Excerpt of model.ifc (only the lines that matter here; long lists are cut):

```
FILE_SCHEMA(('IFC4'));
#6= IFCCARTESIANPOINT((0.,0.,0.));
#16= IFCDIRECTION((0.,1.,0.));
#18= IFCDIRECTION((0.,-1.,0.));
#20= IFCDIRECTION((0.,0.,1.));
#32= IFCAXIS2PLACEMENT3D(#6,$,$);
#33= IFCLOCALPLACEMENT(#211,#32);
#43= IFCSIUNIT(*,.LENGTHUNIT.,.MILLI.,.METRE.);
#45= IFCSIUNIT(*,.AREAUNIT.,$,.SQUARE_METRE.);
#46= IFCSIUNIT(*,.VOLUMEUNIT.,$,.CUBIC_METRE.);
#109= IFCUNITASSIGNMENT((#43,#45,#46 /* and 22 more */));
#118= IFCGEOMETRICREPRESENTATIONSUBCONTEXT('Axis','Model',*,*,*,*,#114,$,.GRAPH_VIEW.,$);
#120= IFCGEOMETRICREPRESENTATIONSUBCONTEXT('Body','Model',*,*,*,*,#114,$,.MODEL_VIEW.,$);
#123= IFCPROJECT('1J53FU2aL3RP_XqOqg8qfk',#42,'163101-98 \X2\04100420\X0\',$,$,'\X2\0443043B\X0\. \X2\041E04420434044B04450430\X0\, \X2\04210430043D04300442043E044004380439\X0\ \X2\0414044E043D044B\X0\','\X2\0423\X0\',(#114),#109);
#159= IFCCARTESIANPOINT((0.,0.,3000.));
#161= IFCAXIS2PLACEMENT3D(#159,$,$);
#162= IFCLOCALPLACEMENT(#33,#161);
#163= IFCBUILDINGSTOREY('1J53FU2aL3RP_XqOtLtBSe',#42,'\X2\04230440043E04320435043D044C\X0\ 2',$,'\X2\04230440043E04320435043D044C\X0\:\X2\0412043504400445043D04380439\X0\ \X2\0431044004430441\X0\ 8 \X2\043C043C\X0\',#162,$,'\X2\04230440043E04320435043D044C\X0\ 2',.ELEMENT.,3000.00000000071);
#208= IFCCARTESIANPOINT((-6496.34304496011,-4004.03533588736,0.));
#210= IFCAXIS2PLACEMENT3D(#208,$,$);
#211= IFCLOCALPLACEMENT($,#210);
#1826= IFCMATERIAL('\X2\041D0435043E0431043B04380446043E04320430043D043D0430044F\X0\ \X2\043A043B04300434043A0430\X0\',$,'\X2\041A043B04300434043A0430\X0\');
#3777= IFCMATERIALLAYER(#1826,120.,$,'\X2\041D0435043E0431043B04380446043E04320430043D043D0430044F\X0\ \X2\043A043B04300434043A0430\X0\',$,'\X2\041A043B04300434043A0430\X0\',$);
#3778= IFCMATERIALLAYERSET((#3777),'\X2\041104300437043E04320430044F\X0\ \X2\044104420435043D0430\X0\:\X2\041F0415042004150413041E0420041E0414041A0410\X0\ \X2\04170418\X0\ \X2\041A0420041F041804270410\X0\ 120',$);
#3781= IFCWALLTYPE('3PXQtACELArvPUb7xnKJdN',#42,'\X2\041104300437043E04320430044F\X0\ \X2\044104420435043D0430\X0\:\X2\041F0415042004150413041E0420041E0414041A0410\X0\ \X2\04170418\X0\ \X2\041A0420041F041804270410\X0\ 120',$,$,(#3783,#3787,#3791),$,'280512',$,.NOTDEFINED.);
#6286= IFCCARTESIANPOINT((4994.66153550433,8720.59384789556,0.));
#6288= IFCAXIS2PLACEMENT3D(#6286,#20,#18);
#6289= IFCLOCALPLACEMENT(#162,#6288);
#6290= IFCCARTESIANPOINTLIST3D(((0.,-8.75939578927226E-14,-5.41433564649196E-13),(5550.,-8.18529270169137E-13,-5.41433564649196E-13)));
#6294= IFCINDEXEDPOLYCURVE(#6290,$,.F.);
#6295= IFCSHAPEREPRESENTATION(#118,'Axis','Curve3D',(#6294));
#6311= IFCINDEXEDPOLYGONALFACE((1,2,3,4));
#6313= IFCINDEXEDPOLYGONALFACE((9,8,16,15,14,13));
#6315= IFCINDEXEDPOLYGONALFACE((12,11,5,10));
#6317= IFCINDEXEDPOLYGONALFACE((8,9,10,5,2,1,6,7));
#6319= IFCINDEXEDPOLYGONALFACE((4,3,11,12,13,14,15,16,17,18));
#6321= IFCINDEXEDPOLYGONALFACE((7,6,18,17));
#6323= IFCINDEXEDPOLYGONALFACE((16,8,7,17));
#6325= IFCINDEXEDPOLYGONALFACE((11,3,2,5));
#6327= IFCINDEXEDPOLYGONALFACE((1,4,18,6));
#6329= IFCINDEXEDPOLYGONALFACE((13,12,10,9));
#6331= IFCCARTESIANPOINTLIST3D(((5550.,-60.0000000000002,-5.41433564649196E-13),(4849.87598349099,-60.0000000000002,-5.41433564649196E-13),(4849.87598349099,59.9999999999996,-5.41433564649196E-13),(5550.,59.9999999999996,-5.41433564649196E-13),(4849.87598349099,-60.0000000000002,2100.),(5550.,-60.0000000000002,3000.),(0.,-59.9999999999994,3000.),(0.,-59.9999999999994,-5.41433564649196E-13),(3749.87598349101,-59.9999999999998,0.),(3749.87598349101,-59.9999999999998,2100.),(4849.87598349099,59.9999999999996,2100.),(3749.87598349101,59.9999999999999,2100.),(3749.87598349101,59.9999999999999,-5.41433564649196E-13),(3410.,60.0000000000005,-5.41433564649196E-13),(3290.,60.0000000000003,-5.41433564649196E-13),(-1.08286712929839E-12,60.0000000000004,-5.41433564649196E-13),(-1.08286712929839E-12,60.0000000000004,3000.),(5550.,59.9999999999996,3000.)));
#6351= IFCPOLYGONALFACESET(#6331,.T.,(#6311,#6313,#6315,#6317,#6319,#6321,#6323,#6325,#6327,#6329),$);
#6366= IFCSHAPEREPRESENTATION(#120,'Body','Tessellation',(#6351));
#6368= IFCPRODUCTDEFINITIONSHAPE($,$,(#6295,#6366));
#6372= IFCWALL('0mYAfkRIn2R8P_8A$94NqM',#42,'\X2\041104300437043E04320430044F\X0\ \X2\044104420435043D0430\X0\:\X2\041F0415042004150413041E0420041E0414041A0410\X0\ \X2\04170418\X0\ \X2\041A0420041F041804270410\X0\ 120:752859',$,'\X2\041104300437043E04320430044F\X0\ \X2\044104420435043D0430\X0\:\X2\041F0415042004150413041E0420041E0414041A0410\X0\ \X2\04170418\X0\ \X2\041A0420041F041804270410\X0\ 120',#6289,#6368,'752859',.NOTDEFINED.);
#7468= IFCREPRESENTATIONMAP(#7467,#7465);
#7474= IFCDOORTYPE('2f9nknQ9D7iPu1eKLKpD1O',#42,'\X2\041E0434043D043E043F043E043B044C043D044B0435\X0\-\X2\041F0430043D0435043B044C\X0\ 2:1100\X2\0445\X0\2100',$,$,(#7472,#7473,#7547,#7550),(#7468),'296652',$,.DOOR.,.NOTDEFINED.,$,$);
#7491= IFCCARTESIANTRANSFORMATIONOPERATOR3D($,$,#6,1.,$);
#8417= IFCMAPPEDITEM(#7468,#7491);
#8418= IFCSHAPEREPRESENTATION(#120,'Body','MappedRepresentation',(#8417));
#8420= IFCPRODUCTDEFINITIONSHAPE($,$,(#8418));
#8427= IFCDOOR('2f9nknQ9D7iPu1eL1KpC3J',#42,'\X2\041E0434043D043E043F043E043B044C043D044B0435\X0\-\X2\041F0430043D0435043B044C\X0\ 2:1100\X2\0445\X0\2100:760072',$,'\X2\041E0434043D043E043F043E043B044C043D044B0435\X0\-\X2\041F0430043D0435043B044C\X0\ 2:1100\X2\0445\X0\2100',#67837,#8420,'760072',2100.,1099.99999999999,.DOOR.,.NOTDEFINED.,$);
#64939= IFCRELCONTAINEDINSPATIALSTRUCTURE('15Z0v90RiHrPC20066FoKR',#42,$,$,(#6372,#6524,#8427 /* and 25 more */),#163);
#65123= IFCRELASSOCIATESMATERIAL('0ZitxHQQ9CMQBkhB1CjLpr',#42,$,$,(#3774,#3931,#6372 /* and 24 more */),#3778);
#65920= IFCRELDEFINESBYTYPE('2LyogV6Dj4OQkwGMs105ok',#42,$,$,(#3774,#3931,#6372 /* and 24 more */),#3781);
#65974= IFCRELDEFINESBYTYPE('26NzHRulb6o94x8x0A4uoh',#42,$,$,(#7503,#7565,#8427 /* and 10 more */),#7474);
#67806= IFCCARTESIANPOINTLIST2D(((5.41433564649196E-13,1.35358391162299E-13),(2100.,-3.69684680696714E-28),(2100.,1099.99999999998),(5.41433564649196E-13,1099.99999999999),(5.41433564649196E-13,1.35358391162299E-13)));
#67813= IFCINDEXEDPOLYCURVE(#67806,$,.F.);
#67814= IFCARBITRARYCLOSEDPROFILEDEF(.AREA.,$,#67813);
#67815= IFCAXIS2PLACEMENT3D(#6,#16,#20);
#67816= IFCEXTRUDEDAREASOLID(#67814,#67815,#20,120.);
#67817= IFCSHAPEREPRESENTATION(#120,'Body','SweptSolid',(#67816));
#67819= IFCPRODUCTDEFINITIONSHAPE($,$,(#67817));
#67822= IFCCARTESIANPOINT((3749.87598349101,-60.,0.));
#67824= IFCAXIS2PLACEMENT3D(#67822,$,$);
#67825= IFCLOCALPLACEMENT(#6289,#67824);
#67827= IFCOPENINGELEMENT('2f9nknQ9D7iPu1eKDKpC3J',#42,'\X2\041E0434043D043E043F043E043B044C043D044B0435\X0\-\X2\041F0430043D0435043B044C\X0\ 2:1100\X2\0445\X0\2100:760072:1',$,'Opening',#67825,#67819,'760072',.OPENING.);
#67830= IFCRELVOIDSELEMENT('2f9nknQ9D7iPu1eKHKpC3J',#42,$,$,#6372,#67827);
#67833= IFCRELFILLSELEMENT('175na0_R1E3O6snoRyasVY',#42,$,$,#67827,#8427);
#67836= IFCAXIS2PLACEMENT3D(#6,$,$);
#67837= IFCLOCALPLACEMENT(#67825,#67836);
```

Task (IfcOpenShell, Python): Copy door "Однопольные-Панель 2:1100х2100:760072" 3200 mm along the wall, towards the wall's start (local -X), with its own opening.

```python
import ifcopenshell
import ifcopenshell.api.feature
import ifcopenshell.api.geometry
import ifcopenshell.api.root
import ifcopenshell.geom
import ifcopenshell.util.element
import ifcopenshell.util.placement
import ifcopenshell.util.shape
import ifcopenshell.util.unit

model = ifcopenshell.open("model.ifc")
unit_scale = ifcopenshell.util.unit.calculate_unit_scale(model)
settings = ifcopenshell.geom.settings()


def volume(element):
    """Net volume in cubic metres, openings subtracted."""
    shape = ifcopenshell.geom.create_shape(settings, element)
    return ifcopenshell.util.shape.get_volume(shape.geometry)


def reuse_history(source, copy):
    """copy_class also copies each property set's owner history, people and application; keep the originals."""
    for rel in copy.IsDefinedBy:
        if rel.is_a("IfcRelDefinesByProperties") and (history := rel.RelatingPropertyDefinition.OwnerHistory):
            rel.RelatingPropertyDefinition.OwnerHistory = source.OwnerHistory
            ifcopenshell.util.element.remove_deep2(model, history)


door = model.by_guid("2f9nknQ9D7iPu1eL1KpC3J")
opening = door.FillsVoids[0].RelatingOpeningElement
wall = opening.VoidsElements[0].RelatingBuildingElement
before = volume(wall)
shift = ifcopenshell.util.placement.get_local_placement(wall.ObjectPlacement)[:3, 0] * -3.2 / unit_scale

# copy_class copies the void relationship, type, container and properties, but no geometry.
new_opening = ifcopenshell.api.root.copy_class(model, product=opening)
new_opening.Representation = ifcopenshell.util.element.copy_deep(
    model, opening.Representation, exclude=["IfcGeometricRepresentationContext", "IfcRepresentationMap"]
)
new_opening.Name = "Однопольные-Панель 2:1100х2100"
new_opening.Tag = None
new_door = ifcopenshell.api.root.copy_class(model, product=door)
new_door.Representation = ifcopenshell.util.element.copy_deep(
    model, door.Representation, exclude=["IfcGeometricRepresentationContext", "IfcRepresentationMap"]
)
new_door.Name = "Однопольные-Панель 2:1100х2100"
new_door.Tag = None
reuse_history(door, new_door)
ifcopenshell.api.feature.add_filling(model, opening=new_opening, element=new_door)

for old, new in ((opening, new_opening), (door, new_door)):
    matrix = ifcopenshell.util.placement.get_local_placement(old.ObjectPlacement)
    matrix[:3, 3] += shift
    ifcopenshell.api.geometry.edit_object_placement(model, product=new, matrix=matrix, is_si=False)

after = volume(wall)

print(f"wall volume {before:.3f} -> {after:.3f} m3")

model.write("model_updated.ifc")
```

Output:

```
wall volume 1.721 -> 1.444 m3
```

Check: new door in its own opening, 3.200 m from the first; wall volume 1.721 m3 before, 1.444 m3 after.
